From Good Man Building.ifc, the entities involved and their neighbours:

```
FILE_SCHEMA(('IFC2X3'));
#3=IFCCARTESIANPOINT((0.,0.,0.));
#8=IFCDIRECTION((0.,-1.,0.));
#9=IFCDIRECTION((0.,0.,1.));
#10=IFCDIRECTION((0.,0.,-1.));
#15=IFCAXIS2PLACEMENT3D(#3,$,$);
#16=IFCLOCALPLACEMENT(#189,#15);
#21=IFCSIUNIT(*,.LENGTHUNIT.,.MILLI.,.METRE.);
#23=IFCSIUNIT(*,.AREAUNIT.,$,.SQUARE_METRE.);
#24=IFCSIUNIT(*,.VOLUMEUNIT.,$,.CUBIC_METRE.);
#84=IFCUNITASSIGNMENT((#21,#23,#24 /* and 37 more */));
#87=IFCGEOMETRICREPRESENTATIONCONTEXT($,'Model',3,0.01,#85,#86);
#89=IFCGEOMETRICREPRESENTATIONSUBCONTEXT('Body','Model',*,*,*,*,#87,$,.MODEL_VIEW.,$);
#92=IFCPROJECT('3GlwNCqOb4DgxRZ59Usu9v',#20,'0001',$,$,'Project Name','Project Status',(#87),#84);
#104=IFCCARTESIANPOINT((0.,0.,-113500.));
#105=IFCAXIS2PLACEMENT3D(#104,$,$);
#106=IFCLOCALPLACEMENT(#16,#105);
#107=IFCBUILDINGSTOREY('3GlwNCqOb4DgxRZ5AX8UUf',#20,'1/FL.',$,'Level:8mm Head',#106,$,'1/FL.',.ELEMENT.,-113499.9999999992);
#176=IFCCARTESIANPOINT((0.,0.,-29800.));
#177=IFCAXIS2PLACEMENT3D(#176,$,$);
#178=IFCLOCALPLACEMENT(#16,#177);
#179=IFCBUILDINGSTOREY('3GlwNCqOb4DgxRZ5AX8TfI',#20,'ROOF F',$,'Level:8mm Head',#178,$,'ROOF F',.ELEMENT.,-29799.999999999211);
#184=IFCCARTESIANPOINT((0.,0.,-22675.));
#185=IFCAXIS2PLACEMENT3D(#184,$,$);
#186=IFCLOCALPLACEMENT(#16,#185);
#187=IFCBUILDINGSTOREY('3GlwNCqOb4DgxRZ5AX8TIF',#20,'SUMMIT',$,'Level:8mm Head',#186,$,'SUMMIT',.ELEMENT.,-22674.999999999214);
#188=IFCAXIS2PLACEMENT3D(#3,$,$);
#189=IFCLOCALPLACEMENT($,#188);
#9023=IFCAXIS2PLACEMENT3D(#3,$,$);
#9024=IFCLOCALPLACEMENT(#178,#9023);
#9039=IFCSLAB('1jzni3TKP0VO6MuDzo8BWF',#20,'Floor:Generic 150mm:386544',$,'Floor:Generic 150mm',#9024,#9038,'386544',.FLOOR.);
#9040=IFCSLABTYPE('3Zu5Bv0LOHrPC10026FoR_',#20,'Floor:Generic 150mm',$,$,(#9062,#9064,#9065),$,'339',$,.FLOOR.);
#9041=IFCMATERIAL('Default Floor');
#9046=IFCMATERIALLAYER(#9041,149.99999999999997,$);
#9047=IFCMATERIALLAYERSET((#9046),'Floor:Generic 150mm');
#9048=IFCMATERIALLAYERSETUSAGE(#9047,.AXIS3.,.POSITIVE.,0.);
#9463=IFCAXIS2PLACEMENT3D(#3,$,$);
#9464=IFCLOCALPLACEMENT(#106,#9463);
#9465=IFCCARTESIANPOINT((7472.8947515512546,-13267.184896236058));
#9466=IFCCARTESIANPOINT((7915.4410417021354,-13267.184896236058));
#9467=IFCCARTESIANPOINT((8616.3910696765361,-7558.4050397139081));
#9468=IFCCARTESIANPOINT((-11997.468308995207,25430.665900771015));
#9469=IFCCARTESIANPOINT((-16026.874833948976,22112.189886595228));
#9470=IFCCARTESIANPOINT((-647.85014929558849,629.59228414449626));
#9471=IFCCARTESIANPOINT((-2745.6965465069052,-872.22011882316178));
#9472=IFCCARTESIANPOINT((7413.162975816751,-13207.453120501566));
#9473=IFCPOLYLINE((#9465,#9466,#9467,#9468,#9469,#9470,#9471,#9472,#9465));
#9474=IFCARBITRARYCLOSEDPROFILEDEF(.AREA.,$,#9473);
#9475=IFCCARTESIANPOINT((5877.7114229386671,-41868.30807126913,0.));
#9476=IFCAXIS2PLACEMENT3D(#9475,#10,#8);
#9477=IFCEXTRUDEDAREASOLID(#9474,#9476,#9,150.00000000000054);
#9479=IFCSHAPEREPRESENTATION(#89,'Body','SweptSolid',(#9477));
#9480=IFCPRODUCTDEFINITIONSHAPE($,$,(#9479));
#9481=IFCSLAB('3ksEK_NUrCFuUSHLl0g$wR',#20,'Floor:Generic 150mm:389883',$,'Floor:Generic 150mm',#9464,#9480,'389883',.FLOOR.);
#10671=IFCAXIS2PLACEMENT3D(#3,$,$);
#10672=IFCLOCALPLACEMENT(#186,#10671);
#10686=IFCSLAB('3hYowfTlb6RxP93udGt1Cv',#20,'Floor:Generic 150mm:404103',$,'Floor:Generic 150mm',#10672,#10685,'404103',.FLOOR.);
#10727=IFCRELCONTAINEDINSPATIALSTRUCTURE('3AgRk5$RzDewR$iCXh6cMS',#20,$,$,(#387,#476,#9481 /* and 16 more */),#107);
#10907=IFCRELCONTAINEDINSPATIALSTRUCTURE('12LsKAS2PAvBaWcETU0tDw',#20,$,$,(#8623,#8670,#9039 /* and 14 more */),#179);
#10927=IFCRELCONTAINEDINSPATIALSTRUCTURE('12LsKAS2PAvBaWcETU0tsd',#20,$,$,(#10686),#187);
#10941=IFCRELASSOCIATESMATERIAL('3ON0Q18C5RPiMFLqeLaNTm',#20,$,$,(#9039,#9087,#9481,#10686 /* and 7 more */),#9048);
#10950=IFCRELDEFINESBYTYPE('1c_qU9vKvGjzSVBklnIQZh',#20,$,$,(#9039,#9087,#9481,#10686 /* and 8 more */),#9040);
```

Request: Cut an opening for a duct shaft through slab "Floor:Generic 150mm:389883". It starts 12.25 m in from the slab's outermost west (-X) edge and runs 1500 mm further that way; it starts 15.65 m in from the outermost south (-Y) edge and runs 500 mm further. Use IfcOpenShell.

```python
import numpy as np
import ifcopenshell
import ifcopenshell.api.feature
import ifcopenshell.api.geometry
import ifcopenshell.api.root
import ifcopenshell.geom
import ifcopenshell.util.placement
import ifcopenshell.util.representation
import ifcopenshell.util.shape
import ifcopenshell.util.unit

model = ifcopenshell.open("Good Man Building.ifc")
unit_scale = ifcopenshell.util.unit.calculate_unit_scale(model)
settings = ifcopenshell.geom.settings()


def volume(element):
    """Net volume in cubic metres, openings subtracted."""
    shape = ifcopenshell.geom.create_shape(settings, element)
    return ifcopenshell.util.shape.get_volume(shape.geometry)


slab = model.by_guid("3ksEK_NUrCFuUSHLl0g$wR")
before = volume(slab)

# Extent in the slab's own axes, in metres. The edges named are its -X and -Y sides.
slab_shape = ifcopenshell.geom.create_shape(settings, slab)
vertices = ifcopenshell.util.shape.get_vertices(slab_shape.geometry)
x_min, y_min, bottom = vertices.min(axis=0)
top = vertices[:, 2].max()

opening = ifcopenshell.api.root.create_entity(model, ifc_class="IfcOpeningElement", name="Duct shaft opening")
context = ifcopenshell.util.representation.get_context(model, "Model", "Body", "MODEL_VIEW")
width, depth = 1.5, 0.5
outline = [(0.0, 0.0), (width, 0.0), (width, depth), (0.0, depth), (0.0, 0.0)]
# Overshoot both faces by 50 mm so the cut is clean.
shape = ifcopenshell.api.geometry.add_slab_representation(
    model, context=context, depth=top - bottom + 0.1, polyline=outline
)
ifcopenshell.api.geometry.assign_representation(model, product=opening, representation=shape)

matrix = ifcopenshell.util.placement.get_local_placement(slab.ObjectPlacement)
matrix[:, 3] = matrix @ np.append(np.array([x_min + 12.25, y_min + 15.65, bottom - 0.05]) / unit_scale, 1.0)
ifcopenshell.api.geometry.edit_object_placement(model, product=opening, matrix=matrix, is_si=False)
ifcopenshell.api.feature.add_feature(model, feature=opening, element=slab)

after = volume(slab)

print(f"slab volume {before:.3f} -> {after:.3f} m3")

model.write("Good Man Building_updated.ifc")
```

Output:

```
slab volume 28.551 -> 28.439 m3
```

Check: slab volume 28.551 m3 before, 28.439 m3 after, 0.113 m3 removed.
